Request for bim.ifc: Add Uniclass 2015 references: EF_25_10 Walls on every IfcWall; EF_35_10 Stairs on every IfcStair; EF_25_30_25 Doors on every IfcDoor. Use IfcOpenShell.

First a look at what the model holds.

```python
import ifcopenshell

model = ifcopenshell.open("bim.ifc")
print(model.schema)
print("classifications:", [c.Name for c in model.by_type("IfcClassification")])
for ifc_class in ("IfcDoor", "IfcRoof", "IfcStair", "IfcWall", "IfcWindow"):
    print(ifc_class, len(model.by_type(ifc_class)))
```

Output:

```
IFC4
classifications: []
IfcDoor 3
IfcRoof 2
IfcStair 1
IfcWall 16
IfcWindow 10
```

```python
import ifcopenshell
import ifcopenshell.api.classification

model = ifcopenshell.open("bim.ifc")

system = ifcopenshell.api.classification.add_classification(model, classification="Uniclass 2015")

codes = {
    "IfcWall": ("EF_25_10", "Walls"),
    "IfcStair": ("EF_35_10", "Stairs"),
    "IfcDoor": ("EF_25_30_25", "Doors"),
}
for ifc_class, (code, name) in codes.items():
    products = model.by_type(ifc_class)
    ifcopenshell.api.classification.add_reference(
        model, products=products, classification=system, identification=code, name=name
    )
    print(code, len(products))

model.write("bim_edited.ifc")
```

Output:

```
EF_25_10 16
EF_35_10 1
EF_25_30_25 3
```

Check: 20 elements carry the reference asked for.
